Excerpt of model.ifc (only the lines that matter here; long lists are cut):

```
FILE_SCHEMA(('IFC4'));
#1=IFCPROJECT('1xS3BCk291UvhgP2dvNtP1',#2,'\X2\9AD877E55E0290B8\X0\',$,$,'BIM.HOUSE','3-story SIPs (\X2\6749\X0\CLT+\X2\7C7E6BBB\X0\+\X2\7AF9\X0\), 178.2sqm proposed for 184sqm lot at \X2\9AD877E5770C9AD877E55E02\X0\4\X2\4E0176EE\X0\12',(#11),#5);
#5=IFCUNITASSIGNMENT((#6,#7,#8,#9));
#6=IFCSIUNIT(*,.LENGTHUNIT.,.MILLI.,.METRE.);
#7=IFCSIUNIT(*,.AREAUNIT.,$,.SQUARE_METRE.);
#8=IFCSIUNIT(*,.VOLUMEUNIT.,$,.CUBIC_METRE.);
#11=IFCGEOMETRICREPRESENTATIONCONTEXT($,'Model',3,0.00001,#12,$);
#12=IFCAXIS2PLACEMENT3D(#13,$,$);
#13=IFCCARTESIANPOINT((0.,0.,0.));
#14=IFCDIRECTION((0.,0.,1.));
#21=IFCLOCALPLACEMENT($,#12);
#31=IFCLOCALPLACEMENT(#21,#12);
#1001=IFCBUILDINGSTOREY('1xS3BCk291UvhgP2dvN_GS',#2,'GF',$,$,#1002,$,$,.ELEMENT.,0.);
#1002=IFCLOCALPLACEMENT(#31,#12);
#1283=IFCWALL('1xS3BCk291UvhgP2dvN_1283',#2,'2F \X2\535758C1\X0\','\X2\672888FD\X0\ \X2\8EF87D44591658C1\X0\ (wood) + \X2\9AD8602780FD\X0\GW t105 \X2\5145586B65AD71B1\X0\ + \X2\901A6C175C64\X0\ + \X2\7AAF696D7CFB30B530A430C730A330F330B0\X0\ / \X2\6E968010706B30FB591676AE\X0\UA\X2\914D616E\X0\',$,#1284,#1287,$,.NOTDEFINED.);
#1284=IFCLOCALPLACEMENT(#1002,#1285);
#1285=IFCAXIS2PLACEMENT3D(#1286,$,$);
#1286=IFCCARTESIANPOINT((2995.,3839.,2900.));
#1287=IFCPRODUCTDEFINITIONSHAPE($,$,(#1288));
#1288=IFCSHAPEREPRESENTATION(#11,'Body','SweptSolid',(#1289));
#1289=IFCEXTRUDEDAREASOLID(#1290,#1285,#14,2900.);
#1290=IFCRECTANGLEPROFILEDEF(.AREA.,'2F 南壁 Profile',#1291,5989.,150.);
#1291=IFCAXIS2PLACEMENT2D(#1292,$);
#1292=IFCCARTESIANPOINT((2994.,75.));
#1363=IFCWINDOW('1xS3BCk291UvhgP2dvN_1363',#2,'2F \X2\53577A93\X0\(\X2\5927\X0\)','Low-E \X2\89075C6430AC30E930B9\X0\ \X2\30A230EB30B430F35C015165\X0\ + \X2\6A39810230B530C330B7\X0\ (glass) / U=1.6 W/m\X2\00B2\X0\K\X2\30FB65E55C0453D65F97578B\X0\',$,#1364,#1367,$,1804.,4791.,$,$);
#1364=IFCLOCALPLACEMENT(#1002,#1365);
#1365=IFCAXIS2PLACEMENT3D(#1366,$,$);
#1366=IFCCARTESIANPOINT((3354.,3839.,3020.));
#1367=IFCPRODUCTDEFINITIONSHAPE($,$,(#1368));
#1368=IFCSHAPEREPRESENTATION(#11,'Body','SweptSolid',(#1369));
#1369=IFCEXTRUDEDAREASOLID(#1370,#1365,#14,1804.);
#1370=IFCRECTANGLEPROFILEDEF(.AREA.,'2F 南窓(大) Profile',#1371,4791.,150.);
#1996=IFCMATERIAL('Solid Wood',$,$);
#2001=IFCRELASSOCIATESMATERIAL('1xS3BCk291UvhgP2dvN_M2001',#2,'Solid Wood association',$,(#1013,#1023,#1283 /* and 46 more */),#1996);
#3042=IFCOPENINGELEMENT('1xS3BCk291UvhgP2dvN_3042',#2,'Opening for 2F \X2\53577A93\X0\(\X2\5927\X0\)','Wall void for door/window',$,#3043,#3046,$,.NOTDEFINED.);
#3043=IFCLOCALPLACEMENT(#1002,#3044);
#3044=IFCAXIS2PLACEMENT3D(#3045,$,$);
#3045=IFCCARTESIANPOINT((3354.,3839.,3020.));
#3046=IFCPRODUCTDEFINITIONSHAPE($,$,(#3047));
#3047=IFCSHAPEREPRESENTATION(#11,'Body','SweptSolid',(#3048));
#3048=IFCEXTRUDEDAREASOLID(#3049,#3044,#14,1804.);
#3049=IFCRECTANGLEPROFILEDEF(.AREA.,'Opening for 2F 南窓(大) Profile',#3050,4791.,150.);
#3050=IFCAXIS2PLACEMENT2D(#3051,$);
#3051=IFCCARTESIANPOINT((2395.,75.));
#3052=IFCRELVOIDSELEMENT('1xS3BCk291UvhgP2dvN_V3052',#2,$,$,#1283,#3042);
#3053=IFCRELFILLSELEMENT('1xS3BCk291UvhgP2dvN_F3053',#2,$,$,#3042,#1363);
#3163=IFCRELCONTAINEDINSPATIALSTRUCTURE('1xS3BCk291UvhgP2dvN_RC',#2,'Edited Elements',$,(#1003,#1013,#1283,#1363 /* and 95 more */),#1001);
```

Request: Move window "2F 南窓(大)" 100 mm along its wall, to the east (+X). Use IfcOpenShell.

```python
import ifcopenshell
import ifcopenshell.api.geometry
import ifcopenshell.util.placement
import ifcopenshell.util.unit

model = ifcopenshell.open("model.ifc")
unit_scale = ifcopenshell.util.unit.calculate_unit_scale(model)

window = model.by_guid("1xS3BCk291UvhgP2dvN_1363")
opening = window.FillsVoids[0].RelatingOpeningElement
wall = opening.VoidsElements[0].RelatingBuildingElement

wall_matrix = ifcopenshell.util.placement.get_local_placement(wall.ObjectPlacement)
shift = wall_matrix[:3, 0] * 0.1 / unit_scale
before = ifcopenshell.util.placement.get_local_placement(window.ObjectPlacement)[:3, 3].copy()

# The window is not placed relative to its opening, so move both.
for product in (opening, window):
    matrix = ifcopenshell.util.placement.get_local_placement(product.ObjectPlacement)
    matrix[:3, 3] += shift
    ifcopenshell.api.geometry.edit_object_placement(model, product=product, matrix=matrix, is_si=False)

after = ifcopenshell.util.placement.get_local_placement(window.ObjectPlacement)[:3, 3]
print("window moved by", (after - before).round(3) + 0.0)

model.write("model_edited.ifc")
```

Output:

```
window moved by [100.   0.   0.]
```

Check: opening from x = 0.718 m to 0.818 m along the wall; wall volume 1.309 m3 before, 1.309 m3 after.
